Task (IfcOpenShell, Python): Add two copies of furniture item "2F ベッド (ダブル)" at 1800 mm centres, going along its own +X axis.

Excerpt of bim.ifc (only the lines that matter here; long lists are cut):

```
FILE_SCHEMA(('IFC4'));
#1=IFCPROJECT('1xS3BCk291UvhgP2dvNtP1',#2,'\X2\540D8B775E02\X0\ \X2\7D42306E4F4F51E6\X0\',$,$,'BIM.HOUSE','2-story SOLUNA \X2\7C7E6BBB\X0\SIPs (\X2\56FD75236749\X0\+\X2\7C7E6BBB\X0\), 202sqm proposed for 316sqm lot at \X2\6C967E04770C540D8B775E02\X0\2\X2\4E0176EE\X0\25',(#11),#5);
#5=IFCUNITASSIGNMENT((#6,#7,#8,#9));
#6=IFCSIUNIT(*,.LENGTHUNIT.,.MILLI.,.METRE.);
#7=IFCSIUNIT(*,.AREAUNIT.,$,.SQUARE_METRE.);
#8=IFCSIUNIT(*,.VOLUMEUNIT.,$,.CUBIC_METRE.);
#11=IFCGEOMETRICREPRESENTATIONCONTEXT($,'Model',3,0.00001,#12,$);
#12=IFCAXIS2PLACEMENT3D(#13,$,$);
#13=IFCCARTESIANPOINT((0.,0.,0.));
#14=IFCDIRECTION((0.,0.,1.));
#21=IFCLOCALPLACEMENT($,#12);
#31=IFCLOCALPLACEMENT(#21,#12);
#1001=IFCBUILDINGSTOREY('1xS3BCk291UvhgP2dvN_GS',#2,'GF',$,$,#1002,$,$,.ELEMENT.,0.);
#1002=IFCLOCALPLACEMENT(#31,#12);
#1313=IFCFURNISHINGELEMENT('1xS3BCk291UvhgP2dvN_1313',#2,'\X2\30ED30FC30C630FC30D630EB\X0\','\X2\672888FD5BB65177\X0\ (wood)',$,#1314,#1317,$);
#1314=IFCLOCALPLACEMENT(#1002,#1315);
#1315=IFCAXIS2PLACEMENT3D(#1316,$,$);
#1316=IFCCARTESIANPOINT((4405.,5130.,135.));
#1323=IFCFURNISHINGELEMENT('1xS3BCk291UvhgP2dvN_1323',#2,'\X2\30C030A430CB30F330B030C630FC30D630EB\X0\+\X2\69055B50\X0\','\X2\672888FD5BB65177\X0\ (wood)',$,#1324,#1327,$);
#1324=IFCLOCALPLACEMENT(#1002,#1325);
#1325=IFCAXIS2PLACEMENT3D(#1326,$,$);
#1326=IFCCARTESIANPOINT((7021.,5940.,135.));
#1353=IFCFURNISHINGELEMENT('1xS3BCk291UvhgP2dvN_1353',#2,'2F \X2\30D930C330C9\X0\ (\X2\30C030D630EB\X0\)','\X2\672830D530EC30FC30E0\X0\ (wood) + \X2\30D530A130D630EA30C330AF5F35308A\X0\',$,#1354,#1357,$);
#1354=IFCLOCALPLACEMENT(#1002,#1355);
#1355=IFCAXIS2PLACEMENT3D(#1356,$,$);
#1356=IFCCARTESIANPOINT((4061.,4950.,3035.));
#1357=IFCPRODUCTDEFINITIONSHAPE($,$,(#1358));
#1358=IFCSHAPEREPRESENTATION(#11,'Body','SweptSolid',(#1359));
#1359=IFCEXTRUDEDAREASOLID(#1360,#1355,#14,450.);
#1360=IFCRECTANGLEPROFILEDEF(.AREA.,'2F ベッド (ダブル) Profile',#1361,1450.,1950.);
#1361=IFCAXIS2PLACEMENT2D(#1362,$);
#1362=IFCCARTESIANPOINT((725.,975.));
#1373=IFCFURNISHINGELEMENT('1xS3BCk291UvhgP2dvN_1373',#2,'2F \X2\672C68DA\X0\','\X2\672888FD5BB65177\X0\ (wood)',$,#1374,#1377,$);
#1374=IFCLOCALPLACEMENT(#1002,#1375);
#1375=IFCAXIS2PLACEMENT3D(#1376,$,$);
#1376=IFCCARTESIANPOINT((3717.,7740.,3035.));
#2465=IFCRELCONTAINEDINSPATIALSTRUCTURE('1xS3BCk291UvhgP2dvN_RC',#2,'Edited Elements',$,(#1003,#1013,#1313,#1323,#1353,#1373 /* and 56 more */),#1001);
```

```python
import ifcopenshell
import ifcopenshell.api.geometry
import ifcopenshell.api.root
import ifcopenshell.util.element
import ifcopenshell.util.placement
import ifcopenshell.util.unit

model = ifcopenshell.open("bim.ifc")
unit_scale = ifcopenshell.util.unit.calculate_unit_scale(model)


def reuse_history(source, copy):
    """copy_class also copies each property set's owner history, people and application; keep the originals."""
    for rel in copy.IsDefinedBy:
        if rel.is_a("IfcRelDefinesByProperties") and (history := rel.RelatingPropertyDefinition.OwnerHistory):
            rel.RelatingPropertyDefinition.OwnerHistory = source.OwnerHistory
            ifcopenshell.util.element.remove_deep2(model, history)


source = model.by_guid("1xS3BCk291UvhgP2dvN_1353")
base = ifcopenshell.util.placement.get_local_placement(source.ObjectPlacement)
step = base[:3, 0] * 1.8 / unit_scale

for i in range(1, 3):
    copy = ifcopenshell.api.root.copy_class(model, product=source)
    copy.Representation = ifcopenshell.util.element.copy_deep(
        model, source.Representation, exclude=["IfcGeometricRepresentationContext", "IfcRepresentationMap"]
    )
    reuse_history(source, copy)
    matrix = base.copy()
    matrix[:3, 3] += i * step
    print("added at", matrix[:3, 3].round(3) + 0.0)
    ifcopenshell.api.geometry.edit_object_placement(model, product=copy, matrix=matrix, is_si=False)

model.write("bim_edited.ifc")
```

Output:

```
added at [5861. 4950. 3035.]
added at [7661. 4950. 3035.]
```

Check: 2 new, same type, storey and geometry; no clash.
